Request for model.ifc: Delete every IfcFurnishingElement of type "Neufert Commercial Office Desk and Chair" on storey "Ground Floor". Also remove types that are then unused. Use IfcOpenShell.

First a look at what the model holds.

```python
import ifcopenshell
import ifcopenshell.util.element

model = ifcopenshell.open("model.ifc")
print(model.schema)
storey = next(s for s in model.by_type("IfcBuildingStorey") if s.Name == "Ground Floor")
furniture = [e for e in ifcopenshell.util.element.get_decomposition(storey) if e.is_a("IfcFurnishingElement")]
seen = {}
for e in furniture:
    element_type = ifcopenshell.util.element.get_type(e)
    name = element_type.Name if element_type not in (None, e) else None
    seen[name] = seen.get(name, 0) + 1
for name, count in sorted(seen.items(), key=str):
    print(count, "x", name)
```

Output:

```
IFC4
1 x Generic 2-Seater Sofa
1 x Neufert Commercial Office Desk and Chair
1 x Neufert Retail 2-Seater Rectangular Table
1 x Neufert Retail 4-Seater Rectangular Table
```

```python
import ifcopenshell
import ifcopenshell.api.root
import ifcopenshell.util.element

model = ifcopenshell.open("model.ifc")

storey = next(s for s in model.by_type("IfcBuildingStorey") if s.Name == "Ground Floor")
furniture = [e for e in ifcopenshell.util.element.get_decomposition(storey) if e.is_a("IfcFurnishingElement")]
targets = [e for e in furniture if (t := ifcopenshell.util.element.get_type(e)) not in (None, e) and t.Name == "Neufert Commercial Office Desk and Chair"]
types = {ifcopenshell.util.element.get_type(e) for e in targets} - {None, *targets}

for e in targets:
    ifcopenshell.api.root.remove_product(model, product=e)
print(len(targets), "removed")

unused = [t for t in types if not ifcopenshell.util.element.get_types(t)]
for t in unused:
    ifcopenshell.api.root.remove_product(model, product=t)
print(len(unused), "unused types removed")

model.write("model-out.ifc")
```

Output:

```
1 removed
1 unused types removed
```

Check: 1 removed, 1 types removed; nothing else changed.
